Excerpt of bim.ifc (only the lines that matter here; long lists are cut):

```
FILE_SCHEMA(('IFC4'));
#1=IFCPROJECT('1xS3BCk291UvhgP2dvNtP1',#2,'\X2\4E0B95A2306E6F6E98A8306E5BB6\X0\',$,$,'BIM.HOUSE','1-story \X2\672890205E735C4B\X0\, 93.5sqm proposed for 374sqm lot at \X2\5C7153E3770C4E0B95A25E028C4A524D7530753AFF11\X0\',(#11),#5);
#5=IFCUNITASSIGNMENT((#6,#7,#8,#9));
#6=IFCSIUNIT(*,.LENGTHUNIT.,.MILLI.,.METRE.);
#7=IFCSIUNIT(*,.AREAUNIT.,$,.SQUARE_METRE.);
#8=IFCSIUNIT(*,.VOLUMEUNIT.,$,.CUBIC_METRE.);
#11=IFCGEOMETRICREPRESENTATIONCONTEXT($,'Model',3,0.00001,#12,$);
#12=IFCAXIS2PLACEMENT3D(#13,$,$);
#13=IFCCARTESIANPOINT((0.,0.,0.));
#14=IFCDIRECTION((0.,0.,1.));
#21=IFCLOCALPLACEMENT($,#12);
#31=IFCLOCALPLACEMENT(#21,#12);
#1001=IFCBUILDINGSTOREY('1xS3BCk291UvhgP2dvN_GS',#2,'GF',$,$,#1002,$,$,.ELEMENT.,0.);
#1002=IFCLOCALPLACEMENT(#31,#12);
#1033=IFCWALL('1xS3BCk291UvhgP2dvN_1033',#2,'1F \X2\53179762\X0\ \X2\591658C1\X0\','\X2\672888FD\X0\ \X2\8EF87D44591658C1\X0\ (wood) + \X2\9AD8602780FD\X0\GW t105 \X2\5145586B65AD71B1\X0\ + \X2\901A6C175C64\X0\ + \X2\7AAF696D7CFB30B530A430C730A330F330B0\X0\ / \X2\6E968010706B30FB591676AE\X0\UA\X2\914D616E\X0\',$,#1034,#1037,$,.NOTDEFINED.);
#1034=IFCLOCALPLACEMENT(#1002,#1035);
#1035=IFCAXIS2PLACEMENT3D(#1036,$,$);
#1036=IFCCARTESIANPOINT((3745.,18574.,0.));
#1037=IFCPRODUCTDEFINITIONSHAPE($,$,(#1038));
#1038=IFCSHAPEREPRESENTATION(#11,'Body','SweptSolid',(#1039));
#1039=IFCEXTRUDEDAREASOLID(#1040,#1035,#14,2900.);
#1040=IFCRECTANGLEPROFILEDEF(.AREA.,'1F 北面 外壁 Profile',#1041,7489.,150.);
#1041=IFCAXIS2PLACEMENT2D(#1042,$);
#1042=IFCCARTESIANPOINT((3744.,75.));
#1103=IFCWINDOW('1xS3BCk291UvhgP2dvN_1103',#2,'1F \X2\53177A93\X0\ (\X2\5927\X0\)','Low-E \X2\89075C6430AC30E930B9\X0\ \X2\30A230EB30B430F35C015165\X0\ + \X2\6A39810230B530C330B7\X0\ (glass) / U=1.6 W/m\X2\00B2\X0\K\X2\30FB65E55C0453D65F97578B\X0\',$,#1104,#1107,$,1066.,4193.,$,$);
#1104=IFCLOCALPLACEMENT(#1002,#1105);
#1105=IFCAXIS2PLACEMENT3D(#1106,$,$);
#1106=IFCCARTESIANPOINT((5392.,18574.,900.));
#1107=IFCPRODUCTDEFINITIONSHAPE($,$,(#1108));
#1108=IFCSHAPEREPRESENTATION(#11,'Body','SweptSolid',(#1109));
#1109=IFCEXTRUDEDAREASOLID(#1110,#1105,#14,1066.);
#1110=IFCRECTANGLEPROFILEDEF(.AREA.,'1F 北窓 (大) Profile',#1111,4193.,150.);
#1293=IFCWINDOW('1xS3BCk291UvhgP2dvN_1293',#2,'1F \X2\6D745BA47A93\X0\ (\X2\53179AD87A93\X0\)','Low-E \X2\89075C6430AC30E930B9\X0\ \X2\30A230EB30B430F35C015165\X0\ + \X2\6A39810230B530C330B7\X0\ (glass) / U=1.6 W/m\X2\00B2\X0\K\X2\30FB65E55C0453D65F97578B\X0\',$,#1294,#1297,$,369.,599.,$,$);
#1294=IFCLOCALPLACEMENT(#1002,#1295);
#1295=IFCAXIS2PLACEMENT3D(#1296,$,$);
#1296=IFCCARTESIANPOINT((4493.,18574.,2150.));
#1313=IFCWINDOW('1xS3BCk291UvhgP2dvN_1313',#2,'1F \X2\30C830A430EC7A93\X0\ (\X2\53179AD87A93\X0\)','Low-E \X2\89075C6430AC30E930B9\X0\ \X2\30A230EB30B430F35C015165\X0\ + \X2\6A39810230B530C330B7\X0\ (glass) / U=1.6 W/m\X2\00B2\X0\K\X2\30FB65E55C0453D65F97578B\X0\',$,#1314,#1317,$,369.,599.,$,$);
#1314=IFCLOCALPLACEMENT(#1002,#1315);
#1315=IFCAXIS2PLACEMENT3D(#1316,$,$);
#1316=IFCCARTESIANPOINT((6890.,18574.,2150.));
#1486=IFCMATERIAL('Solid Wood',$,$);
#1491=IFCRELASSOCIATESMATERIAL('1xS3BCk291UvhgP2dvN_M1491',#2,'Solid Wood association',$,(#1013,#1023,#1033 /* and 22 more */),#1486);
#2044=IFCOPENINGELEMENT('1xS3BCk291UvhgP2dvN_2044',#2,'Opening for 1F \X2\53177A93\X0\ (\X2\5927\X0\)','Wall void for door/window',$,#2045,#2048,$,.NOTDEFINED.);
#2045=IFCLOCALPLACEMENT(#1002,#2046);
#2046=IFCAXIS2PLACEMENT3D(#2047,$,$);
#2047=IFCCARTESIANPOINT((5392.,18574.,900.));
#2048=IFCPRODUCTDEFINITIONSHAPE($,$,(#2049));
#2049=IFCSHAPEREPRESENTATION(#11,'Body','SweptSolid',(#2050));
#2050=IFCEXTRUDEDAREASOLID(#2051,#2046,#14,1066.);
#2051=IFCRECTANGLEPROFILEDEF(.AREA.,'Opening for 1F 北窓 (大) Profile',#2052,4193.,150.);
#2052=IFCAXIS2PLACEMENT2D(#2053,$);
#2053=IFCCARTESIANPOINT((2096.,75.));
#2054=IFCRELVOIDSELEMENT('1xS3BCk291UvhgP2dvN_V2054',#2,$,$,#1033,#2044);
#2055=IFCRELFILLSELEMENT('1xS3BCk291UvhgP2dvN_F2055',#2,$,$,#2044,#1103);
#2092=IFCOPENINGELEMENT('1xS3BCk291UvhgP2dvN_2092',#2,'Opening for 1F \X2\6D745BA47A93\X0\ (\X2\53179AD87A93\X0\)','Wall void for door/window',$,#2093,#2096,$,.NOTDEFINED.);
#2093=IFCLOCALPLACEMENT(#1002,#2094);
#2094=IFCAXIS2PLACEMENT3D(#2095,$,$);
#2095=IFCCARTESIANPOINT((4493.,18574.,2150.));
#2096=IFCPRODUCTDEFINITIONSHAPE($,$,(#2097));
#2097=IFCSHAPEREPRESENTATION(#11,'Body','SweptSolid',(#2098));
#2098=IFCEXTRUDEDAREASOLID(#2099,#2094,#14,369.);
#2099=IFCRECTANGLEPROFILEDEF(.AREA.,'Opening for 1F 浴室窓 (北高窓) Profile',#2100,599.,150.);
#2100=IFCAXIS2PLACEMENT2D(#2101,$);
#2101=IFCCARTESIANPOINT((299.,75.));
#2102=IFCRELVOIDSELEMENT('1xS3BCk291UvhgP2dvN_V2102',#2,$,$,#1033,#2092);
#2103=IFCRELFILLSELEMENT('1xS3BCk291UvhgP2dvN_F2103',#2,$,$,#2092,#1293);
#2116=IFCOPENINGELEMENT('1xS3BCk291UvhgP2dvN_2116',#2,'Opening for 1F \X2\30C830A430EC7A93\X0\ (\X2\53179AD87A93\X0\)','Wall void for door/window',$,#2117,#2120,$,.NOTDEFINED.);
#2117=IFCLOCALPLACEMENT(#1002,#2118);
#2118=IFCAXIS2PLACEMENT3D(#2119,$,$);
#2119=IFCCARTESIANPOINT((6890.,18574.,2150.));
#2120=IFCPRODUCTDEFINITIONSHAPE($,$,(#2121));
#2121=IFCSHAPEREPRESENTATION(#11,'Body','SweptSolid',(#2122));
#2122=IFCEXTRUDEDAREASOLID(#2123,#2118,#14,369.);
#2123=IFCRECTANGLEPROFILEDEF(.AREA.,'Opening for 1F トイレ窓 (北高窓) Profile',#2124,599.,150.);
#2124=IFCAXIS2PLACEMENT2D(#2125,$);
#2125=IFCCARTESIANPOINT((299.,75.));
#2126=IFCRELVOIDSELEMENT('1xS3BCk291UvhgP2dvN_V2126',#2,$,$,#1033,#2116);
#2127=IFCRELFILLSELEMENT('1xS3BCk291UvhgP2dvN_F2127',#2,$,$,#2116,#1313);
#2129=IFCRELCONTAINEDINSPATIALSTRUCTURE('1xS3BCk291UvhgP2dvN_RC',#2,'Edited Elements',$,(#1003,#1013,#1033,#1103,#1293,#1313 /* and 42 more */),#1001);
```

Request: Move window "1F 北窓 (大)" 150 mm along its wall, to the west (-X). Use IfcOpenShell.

```python
import ifcopenshell
import ifcopenshell.api.geometry
import ifcopenshell.util.placement
import ifcopenshell.util.unit

model = ifcopenshell.open("bim.ifc")
unit_scale = ifcopenshell.util.unit.calculate_unit_scale(model)

window = model.by_guid("1xS3BCk291UvhgP2dvN_1103")
opening = window.FillsVoids[0].RelatingOpeningElement
wall = opening.VoidsElements[0].RelatingBuildingElement

wall_matrix = ifcopenshell.util.placement.get_local_placement(wall.ObjectPlacement)
shift = wall_matrix[:3, 0] * -0.15 / unit_scale
before = ifcopenshell.util.placement.get_local_placement(window.ObjectPlacement)[:3, 3].copy()

# The window is not placed relative to its opening, so move both.
for product in (opening, window):
    matrix = ifcopenshell.util.placement.get_local_placement(product.ObjectPlacement)
    matrix[:3, 3] += shift
    ifcopenshell.api.geometry.edit_object_placement(model, product=product, matrix=matrix, is_si=False)

after = ifcopenshell.util.placement.get_local_placement(window.ObjectPlacement)[:3, 3]
print("window moved by", (after - before).round(3) + 0.0)

model.write("bim_rev.ifc")
```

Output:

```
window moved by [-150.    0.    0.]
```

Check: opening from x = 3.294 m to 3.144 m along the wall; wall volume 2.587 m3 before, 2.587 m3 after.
